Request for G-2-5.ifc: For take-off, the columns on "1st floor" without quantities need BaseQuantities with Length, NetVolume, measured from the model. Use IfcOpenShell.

First a look at what the model holds.

```python
import ifcopenshell
import ifcopenshell.util.element
import ifcopenshell.util.unit

model = ifcopenshell.open("G-2-5.ifc")
print(model.schema)
for unit_type in ("LENGTHUNIT", "AREAUNIT", "VOLUMEUNIT"):
    print(unit_type, ifcopenshell.util.unit.calculate_unit_scale(model, unit_type))
storey = next(s for s in model.by_type("IfcBuildingStorey") if s.Name == "1st floor")
columns = [e for e in ifcopenshell.util.element.get_decomposition(storey) if e.is_a("IfcColumn")]
for e in sorted(columns, key=lambda e: e.id()):
    print(e.id(), e.is_a(), e.Name, list(ifcopenshell.util.element.get_psets(e, qtos_only=True)), sep=" | ")
```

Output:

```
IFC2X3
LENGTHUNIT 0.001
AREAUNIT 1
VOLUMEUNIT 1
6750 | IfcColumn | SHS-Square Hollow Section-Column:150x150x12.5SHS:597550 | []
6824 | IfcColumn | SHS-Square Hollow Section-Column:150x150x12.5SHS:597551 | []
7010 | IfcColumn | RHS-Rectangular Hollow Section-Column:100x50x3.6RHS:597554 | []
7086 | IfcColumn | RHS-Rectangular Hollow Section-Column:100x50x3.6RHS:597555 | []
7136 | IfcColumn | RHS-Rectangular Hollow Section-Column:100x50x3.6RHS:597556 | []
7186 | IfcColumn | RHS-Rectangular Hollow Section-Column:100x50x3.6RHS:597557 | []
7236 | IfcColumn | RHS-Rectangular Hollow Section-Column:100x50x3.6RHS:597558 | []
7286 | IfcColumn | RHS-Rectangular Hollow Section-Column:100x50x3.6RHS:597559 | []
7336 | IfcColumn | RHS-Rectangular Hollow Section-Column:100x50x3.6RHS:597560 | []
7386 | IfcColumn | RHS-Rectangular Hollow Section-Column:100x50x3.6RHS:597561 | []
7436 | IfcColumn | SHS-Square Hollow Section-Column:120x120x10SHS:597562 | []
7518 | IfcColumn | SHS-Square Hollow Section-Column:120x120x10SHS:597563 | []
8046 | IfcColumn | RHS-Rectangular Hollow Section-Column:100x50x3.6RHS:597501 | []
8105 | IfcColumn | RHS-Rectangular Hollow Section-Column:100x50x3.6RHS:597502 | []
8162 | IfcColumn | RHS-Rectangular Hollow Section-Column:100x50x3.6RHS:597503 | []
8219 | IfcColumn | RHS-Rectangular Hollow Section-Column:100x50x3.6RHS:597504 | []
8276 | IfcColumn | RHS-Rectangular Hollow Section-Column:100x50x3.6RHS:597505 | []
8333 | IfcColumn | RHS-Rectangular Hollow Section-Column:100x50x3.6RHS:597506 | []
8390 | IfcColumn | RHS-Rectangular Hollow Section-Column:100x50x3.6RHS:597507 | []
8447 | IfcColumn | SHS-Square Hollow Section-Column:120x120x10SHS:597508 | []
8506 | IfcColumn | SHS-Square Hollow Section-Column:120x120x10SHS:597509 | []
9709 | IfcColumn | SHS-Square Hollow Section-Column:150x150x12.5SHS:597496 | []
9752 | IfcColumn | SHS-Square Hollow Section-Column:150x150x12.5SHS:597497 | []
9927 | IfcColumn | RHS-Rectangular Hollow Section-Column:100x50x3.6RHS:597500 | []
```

```python
import ifcopenshell
import ifcopenshell.api.pset
import ifcopenshell.geom
import ifcopenshell.util.element
import ifcopenshell.util.shape
import ifcopenshell.util.unit

model = ifcopenshell.open("G-2-5.ifc")
unit_scale = ifcopenshell.util.unit.calculate_unit_scale(model)
volume_scale = ifcopenshell.util.unit.calculate_unit_scale(model, "VOLUMEUNIT")
settings = ifcopenshell.geom.settings()

storey = next(s for s in model.by_type("IfcBuildingStorey") if s.Name == "1st floor")
columns = [e for e in ifcopenshell.util.element.get_decomposition(storey) if e.is_a("IfcColumn")]

for e in sorted(columns, key=lambda e: e.id()):
    if ifcopenshell.util.element.get_psets(e, qtos_only=True, should_inherit=False):
        continue
    # Geometry comes back in metres, in the element's own axes.
    shape = ifcopenshell.geom.create_shape(settings, e)
    values = {
        "Length": ifcopenshell.util.shape.get_z(shape.geometry) / unit_scale,
        "NetVolume": ifcopenshell.util.shape.get_volume(shape.geometry) / volume_scale,
    }
    qto = ifcopenshell.api.pset.add_qto(model, product=e, name="BaseQuantities")
    ifcopenshell.api.pset.edit_qto(model, qto=qto, properties=values)
    print(e.id(), {k: round(v, 3) for k, v in values.items()})

model.write("G-2-5-out.ifc")
```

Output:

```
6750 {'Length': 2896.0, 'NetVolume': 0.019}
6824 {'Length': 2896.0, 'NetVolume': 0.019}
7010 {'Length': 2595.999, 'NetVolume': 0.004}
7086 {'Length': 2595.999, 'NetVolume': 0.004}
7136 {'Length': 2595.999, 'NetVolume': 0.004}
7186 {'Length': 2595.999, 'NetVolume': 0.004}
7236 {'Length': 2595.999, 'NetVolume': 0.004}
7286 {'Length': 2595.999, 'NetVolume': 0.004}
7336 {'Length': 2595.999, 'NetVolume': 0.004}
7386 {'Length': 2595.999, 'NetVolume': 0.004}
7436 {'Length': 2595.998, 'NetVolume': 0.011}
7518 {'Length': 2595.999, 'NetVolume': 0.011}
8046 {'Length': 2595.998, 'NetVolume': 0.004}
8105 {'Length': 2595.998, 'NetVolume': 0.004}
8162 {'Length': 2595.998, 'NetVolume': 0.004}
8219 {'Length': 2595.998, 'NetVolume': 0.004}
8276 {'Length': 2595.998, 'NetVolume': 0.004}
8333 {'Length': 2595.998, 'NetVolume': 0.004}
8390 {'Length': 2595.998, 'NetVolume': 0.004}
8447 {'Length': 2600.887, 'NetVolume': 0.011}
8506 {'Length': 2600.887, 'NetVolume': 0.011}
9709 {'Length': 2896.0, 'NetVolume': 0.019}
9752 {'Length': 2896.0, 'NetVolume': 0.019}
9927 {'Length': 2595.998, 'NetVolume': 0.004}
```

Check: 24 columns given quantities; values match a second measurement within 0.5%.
